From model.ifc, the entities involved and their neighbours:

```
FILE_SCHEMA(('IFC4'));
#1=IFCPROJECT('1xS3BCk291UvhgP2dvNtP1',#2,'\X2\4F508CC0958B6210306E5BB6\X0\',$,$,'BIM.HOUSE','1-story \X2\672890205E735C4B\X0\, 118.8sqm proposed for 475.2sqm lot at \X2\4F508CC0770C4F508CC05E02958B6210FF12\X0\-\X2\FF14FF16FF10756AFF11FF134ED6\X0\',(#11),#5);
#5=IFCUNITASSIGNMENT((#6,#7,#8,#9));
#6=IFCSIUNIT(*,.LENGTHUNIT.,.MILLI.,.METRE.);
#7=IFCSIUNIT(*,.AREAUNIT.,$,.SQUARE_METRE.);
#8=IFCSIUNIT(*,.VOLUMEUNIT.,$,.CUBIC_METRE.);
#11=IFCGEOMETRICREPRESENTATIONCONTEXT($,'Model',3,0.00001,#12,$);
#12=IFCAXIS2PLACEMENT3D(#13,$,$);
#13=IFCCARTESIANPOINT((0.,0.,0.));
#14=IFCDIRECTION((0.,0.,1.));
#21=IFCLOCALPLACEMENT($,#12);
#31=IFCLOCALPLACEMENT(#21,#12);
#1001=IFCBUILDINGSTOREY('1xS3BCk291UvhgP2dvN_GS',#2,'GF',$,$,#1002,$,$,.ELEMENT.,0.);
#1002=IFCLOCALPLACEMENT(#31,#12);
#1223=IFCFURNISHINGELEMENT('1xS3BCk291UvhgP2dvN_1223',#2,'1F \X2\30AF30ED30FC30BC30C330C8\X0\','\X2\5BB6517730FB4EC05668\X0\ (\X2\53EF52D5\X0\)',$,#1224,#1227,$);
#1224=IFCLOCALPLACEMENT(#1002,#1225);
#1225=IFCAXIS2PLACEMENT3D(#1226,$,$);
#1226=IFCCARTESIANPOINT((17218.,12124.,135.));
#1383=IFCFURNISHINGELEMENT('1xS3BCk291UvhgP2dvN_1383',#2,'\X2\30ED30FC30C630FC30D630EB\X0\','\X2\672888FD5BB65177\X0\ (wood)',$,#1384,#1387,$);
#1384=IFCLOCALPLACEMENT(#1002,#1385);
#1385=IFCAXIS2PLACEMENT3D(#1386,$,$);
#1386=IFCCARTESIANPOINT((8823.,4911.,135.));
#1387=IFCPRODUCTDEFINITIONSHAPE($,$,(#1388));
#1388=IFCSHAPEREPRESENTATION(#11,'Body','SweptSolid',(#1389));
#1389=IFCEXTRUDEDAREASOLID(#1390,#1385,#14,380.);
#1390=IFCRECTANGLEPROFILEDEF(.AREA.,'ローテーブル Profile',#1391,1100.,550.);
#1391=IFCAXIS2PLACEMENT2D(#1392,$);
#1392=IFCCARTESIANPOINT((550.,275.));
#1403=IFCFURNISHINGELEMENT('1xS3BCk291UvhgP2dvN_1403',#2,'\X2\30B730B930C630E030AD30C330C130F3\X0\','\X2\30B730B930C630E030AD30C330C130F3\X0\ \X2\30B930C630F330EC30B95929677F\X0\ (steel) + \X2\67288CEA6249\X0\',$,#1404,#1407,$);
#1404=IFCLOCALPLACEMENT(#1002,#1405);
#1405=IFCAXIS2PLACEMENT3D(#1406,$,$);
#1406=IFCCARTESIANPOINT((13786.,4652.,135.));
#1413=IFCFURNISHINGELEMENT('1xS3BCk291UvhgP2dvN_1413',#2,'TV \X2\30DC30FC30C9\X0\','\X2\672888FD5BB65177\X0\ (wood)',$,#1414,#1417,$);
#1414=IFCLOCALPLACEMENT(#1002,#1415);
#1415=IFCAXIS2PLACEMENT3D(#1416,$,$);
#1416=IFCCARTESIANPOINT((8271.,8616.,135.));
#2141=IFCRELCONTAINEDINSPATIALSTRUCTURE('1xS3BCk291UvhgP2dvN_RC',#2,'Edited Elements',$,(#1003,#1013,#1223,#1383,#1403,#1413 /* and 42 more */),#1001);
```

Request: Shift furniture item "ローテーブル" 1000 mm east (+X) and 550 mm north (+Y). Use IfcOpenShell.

```python
import ifcopenshell
import ifcopenshell.api.geometry
import ifcopenshell.util.placement

model = ifcopenshell.open("model.ifc")

item = model.by_guid("1xS3BCk291UvhgP2dvN_1383")
matrix = ifcopenshell.util.placement.get_local_placement(item.ObjectPlacement)
matrix[0, 3] += 1000.0
matrix[1, 3] += 550.0
ifcopenshell.api.geometry.edit_object_placement(model, product=item, matrix=matrix, is_si=False)

print(ifcopenshell.util.placement.get_local_placement(item.ObjectPlacement).round(3) + 0.0)

model.write("model_rev.ifc")
```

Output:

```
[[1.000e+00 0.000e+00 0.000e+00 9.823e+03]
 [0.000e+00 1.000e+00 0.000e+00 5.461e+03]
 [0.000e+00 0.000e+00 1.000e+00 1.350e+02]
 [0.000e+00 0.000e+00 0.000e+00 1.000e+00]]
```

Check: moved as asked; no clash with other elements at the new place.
